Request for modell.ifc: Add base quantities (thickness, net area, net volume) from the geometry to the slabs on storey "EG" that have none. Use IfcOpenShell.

First a look at what the model holds.

```python
import ifcopenshell
import ifcopenshell.util.element
import ifcopenshell.util.unit

model = ifcopenshell.open("modell.ifc")
print(model.schema)
for unit_type in ("LENGTHUNIT", "AREAUNIT", "VOLUMEUNIT"):
    print(unit_type, ifcopenshell.util.unit.calculate_unit_scale(model, unit_type))
storey = next(s for s in model.by_type("IfcBuildingStorey") if s.Name == "EG")
slabs = [e for e in ifcopenshell.util.element.get_decomposition(storey) if e.is_a("IfcSlab")]
for e in sorted(slabs, key=lambda e: e.id()):
    print(e.id(), e.is_a(), e.Name, list(ifcopenshell.util.element.get_psets(e, qtos_only=True)), sep=" | ")
```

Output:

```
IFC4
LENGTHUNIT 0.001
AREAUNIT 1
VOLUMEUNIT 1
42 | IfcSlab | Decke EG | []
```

```python
import ifcopenshell
import ifcopenshell.api.pset
import ifcopenshell.geom
import ifcopenshell.util.element
import ifcopenshell.util.shape
import ifcopenshell.util.unit

model = ifcopenshell.open("modell.ifc")
unit_scale = ifcopenshell.util.unit.calculate_unit_scale(model)
area_scale = ifcopenshell.util.unit.calculate_unit_scale(model, "AREAUNIT")
volume_scale = ifcopenshell.util.unit.calculate_unit_scale(model, "VOLUMEUNIT")
settings = ifcopenshell.geom.settings()

storey = next(s for s in model.by_type("IfcBuildingStorey") if s.Name == "EG")
slabs = [e for e in ifcopenshell.util.element.get_decomposition(storey) if e.is_a("IfcSlab")]

for e in sorted(slabs, key=lambda e: e.id()):
    if ifcopenshell.util.element.get_psets(e, qtos_only=True, should_inherit=False):
        continue
    # Geometry comes back in metres, in the element's own axes.
    shape = ifcopenshell.geom.create_shape(settings, e)
    values = {
        "Width": ifcopenshell.util.shape.get_z(shape.geometry) / unit_scale,
        "NetArea": ifcopenshell.util.shape.get_footprint_area(shape.geometry) / area_scale,
        "NetVolume": ifcopenshell.util.shape.get_volume(shape.geometry) / volume_scale,
    }
    qto = ifcopenshell.api.pset.add_qto(model, product=e, name="Qto_SlabBaseQuantities")
    ifcopenshell.api.pset.edit_qto(model, qto=qto, properties=values)
    print(e.id(), {k: round(v, 3) for k, v in values.items()})

model.write("modell-out.ifc")
```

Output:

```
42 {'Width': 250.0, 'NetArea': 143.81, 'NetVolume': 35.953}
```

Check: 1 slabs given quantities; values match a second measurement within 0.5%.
